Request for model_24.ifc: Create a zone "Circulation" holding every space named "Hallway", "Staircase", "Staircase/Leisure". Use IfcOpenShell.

First a look at what the model holds.

```python
import ifcopenshell

model = ifcopenshell.open("model_24.ifc")
print(model.schema)
seen = {}
for space in model.by_type("IfcSpace"):
    seen[space.LongName] = seen.get(space.LongName, 0) + 1
for name, count in sorted(seen.items(), key=str):
    print(count, "x", name)
print("zones:", [z.Name for z in model.by_type("IfcZone")][:20])
```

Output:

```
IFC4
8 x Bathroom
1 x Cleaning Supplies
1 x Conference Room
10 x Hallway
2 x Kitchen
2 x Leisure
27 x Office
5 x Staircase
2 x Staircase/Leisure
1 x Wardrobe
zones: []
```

```python
import ifcopenshell
import ifcopenshell.api.group
import ifcopenshell.api.root

model = ifcopenshell.open("model_24.ifc")

names = {"Hallway", "Staircase", "Staircase/Leisure"}
spaces = [s for s in model.by_type("IfcSpace") if s.LongName in names]

zone = ifcopenshell.api.root.create_entity(model, ifc_class="IfcZone", name="Circulation")
ifcopenshell.api.group.assign_group(model, products=spaces, group=zone)
print(len(spaces), "spaces in", zone.Name)

model.write("model_24_edited.ifc")
```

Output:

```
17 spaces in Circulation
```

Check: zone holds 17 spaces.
